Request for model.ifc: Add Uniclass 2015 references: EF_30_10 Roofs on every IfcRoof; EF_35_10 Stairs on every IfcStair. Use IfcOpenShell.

First a look at what the model holds.

```python
import ifcopenshell

model = ifcopenshell.open("model.ifc")
print(model.schema)
print("classifications:", [c.Name for c in model.by_type("IfcClassification")])
for ifc_class in ("IfcDoor", "IfcRoof", "IfcStair", "IfcWall", "IfcWindow"):
    print(ifc_class, len(model.by_type(ifc_class)))
```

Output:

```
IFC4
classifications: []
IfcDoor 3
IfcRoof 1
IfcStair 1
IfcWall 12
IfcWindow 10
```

```python
import ifcopenshell
import ifcopenshell.api.classification

model = ifcopenshell.open("model.ifc")

system = ifcopenshell.api.classification.add_classification(model, classification="Uniclass 2015")

codes = {
    "IfcRoof": ("EF_30_10", "Roofs"),
    "IfcStair": ("EF_35_10", "Stairs"),
}
for ifc_class, (code, name) in codes.items():
    products = model.by_type(ifc_class)
    ifcopenshell.api.classification.add_reference(
        model, products=products, classification=system, identification=code, name=name
    )
    print(code, len(products))

model.write("model_v2.ifc")
```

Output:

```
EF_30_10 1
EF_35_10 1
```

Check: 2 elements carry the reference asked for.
